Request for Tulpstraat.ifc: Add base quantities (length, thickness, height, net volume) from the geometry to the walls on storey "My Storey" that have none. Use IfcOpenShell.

First a look at what the model holds.

```python
import ifcopenshell
import ifcopenshell.util.element
import ifcopenshell.util.unit

model = ifcopenshell.open("Tulpstraat.ifc")
print(model.schema)
for unit_type in ("LENGTHUNIT", "AREAUNIT", "VOLUMEUNIT"):
    print(unit_type, ifcopenshell.util.unit.calculate_unit_scale(model, unit_type))
storey = next(s for s in model.by_type("IfcBuildingStorey") if s.Name == "My Storey")
walls = [e for e in ifcopenshell.util.element.get_decomposition(storey) if e.is_a("IfcWall")]
for e in sorted(walls, key=lambda e: e.id()):
    print(e.id(), e.is_a(), e.Name, list(ifcopenshell.util.element.get_psets(e, qtos_only=True)), sep=" | ")
```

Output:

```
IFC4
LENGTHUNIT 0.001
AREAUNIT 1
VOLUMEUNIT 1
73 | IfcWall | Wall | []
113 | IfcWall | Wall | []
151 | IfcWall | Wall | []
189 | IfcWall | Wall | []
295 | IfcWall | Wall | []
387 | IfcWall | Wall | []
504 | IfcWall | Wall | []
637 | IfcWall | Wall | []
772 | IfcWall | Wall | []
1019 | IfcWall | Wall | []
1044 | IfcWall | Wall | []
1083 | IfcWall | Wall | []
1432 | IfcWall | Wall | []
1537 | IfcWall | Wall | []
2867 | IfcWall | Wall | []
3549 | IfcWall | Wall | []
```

```python
import ifcopenshell
import ifcopenshell.api.pset
import ifcopenshell.geom
import ifcopenshell.util.element
import ifcopenshell.util.shape
import ifcopenshell.util.unit

model = ifcopenshell.open("Tulpstraat.ifc")
unit_scale = ifcopenshell.util.unit.calculate_unit_scale(model)
volume_scale = ifcopenshell.util.unit.calculate_unit_scale(model, "VOLUMEUNIT")
settings = ifcopenshell.geom.settings()

storey = next(s for s in model.by_type("IfcBuildingStorey") if s.Name == "My Storey")
walls = [e for e in ifcopenshell.util.element.get_decomposition(storey) if e.is_a("IfcWall")]

for e in sorted(walls, key=lambda e: e.id()):
    if ifcopenshell.util.element.get_psets(e, qtos_only=True, should_inherit=False):
        continue
    # Geometry comes back in metres, in the element's own axes.
    shape = ifcopenshell.geom.create_shape(settings, e)
    values = {
        "Length": ifcopenshell.util.shape.get_x(shape.geometry) / unit_scale,
        "Width": ifcopenshell.util.shape.get_y(shape.geometry) / unit_scale,
        "Height": ifcopenshell.util.shape.get_z(shape.geometry) / unit_scale,
        "NetVolume": ifcopenshell.util.shape.get_volume(shape.geometry) / volume_scale,
    }
    qto = ifcopenshell.api.pset.add_qto(model, product=e, name="Qto_WallBaseQuantities")
    ifcopenshell.api.pset.edit_qto(model, qto=qto, properties=values)
    print(e.id(), {k: round(v, 3) for k, v in values.items()})

model.write("Tulpstraat_updated.ifc")
```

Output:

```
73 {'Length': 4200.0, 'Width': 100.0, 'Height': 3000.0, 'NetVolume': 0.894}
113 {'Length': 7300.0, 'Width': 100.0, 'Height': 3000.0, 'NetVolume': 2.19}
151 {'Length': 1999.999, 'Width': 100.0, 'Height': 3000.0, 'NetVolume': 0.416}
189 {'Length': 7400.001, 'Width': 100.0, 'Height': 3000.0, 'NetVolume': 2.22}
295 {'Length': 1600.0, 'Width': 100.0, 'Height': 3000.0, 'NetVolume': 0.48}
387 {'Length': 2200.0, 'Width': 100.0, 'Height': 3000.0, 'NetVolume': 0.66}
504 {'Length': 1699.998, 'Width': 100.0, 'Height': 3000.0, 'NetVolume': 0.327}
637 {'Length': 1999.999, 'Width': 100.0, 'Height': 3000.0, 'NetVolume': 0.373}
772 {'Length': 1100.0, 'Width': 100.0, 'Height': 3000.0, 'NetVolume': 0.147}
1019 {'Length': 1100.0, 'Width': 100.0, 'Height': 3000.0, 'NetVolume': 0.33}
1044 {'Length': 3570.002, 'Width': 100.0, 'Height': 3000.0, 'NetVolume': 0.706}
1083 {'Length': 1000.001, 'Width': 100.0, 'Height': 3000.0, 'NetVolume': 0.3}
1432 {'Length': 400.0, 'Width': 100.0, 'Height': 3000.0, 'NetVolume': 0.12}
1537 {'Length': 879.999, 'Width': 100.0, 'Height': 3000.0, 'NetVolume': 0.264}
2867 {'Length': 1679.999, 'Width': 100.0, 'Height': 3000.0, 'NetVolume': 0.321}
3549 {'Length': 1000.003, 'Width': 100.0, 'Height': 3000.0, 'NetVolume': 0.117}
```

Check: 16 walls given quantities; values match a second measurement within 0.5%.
